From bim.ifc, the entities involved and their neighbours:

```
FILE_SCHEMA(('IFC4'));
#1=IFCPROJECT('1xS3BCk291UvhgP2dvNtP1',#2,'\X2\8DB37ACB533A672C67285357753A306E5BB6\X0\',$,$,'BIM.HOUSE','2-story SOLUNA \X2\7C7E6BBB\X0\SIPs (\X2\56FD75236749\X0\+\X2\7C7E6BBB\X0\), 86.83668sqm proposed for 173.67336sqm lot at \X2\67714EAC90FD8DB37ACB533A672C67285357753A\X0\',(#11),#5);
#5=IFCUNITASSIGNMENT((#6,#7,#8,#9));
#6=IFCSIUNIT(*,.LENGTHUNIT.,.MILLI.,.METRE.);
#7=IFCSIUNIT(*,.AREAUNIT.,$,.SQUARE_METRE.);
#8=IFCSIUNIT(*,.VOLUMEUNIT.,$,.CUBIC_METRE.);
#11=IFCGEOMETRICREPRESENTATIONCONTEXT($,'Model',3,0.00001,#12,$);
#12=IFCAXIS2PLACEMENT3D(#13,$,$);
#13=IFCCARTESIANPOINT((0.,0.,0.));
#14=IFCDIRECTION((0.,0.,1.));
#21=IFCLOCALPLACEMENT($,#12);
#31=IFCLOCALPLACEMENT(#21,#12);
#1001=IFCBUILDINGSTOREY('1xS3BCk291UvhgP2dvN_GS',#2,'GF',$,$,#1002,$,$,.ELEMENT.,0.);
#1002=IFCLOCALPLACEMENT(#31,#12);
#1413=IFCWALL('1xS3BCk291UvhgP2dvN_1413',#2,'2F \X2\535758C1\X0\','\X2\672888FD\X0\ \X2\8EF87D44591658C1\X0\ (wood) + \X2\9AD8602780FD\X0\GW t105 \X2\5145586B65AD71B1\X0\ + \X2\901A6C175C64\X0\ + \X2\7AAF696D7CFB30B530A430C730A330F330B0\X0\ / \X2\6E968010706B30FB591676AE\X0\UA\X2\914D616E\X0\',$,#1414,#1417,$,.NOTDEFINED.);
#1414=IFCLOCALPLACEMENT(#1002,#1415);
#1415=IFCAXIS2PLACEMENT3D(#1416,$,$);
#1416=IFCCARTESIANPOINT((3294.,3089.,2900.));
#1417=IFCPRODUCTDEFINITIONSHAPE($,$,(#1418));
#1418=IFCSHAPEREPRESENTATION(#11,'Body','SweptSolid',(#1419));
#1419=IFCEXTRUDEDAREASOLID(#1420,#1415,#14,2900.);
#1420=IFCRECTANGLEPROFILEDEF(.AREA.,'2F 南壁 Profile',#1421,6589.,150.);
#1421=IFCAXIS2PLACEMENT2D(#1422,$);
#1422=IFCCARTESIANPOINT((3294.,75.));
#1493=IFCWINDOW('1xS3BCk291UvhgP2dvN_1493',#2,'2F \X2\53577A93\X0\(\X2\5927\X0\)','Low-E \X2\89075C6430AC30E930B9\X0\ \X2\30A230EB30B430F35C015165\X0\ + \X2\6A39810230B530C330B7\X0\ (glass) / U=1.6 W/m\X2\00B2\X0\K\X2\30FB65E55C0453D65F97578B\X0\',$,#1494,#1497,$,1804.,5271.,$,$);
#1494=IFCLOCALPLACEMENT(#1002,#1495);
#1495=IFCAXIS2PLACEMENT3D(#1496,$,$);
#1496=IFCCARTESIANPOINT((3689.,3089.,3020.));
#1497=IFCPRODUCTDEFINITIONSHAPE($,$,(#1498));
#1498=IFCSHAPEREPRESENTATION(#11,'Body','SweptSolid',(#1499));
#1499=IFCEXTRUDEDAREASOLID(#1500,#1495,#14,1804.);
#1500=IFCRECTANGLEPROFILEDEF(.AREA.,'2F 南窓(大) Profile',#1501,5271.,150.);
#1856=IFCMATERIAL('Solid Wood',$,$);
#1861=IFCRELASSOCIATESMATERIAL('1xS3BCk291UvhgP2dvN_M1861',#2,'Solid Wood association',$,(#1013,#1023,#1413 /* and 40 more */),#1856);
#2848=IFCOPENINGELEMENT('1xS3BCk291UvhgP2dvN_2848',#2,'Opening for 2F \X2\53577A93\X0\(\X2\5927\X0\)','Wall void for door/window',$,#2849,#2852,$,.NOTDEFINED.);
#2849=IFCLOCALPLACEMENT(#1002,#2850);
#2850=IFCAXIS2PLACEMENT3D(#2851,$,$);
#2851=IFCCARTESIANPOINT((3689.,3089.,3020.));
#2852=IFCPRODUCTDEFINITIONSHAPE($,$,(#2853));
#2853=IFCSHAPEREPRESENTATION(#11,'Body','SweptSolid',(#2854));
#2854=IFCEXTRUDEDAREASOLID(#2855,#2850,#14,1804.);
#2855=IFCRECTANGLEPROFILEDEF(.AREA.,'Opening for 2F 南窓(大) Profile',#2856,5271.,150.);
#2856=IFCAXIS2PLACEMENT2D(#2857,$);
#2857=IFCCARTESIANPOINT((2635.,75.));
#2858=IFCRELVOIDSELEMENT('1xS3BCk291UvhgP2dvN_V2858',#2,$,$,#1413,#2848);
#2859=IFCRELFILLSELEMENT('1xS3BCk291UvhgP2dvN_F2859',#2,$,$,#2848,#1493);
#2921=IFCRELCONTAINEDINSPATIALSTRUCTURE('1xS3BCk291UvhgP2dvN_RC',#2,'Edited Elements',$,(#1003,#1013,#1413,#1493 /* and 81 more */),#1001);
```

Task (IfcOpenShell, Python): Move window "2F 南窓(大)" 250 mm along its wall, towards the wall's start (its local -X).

```python
import ifcopenshell
import ifcopenshell.api.geometry
import ifcopenshell.util.placement
import ifcopenshell.util.unit

model = ifcopenshell.open("bim.ifc")
unit_scale = ifcopenshell.util.unit.calculate_unit_scale(model)

window = model.by_id(1493)
opening = window.FillsVoids[0].RelatingOpeningElement
wall = opening.VoidsElements[0].RelatingBuildingElement

wall_matrix = ifcopenshell.util.placement.get_local_placement(wall.ObjectPlacement)
shift = wall_matrix[:3, 0] * -0.25 / unit_scale
before = ifcopenshell.util.placement.get_local_placement(window.ObjectPlacement)[:3, 3].copy()

# The window is not placed relative to its opening, so move both.
for product in (opening, window):
    matrix = ifcopenshell.util.placement.get_local_placement(product.ObjectPlacement)
    matrix[:3, 3] += shift
    ifcopenshell.api.geometry.edit_object_placement(model, product=product, matrix=matrix, is_si=False)

after = ifcopenshell.util.placement.get_local_placement(window.ObjectPlacement)[:3, 3]
print("window moved by", (after - before).round(3) + 0.0)

model.write("bim-out.ifc")
```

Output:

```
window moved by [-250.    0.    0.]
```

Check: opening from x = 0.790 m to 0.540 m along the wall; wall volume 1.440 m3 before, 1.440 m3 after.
